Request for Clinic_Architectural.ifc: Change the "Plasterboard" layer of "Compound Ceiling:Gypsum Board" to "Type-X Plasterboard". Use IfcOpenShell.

First a look at what the model holds.

```python
import ifcopenshell
import ifcopenshell.util.element

model = ifcopenshell.open("Clinic_Architectural.ifc")
print(model.schema)
for layer_set in model.by_type("IfcMaterialLayerSet"):
    if layer_set.LayerSetName == "Compound Ceiling:Gypsum Board":
        for layer in layer_set.MaterialLayers:
            print(layer.id(), layer.Material and layer.Material.Name, layer.LayerThickness, sep=" | ")
        print(len(ifcopenshell.util.element.get_elements_by_material(model, layer_set)), "elements and types use it")
print(sorted(m.Name for m in model.by_type("IfcMaterial") if m.Name)[:60])
```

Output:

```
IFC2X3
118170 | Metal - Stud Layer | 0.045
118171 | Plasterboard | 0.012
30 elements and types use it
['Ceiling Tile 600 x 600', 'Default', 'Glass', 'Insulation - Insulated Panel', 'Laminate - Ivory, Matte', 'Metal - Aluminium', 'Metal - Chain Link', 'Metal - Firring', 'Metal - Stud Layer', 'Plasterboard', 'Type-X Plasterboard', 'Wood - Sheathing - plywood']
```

```python
import ifcopenshell
import ifcopenshell.api.material

model = ifcopenshell.open("Clinic_Architectural.ifc")

layer_set = next(s for s in model.by_type("IfcMaterialLayerSet") if s.LayerSetName == "Compound Ceiling:Gypsum Board")
layer = next(l for l in layer_set.MaterialLayers if l.Material and l.Material.Name == "Plasterboard")
material = next(m for m in model.by_type("IfcMaterial") if m.Name == "Type-X Plasterboard")

# Point this one layer at the other material; renaming the old one would change it everywhere.
ifcopenshell.api.material.edit_layer(model, layer=layer, attributes={}, material=material)

print([l.Material.Name if l.Material else None for l in layer_set.MaterialLayers])

model.write("Clinic_Architectural_v2.ifc")
```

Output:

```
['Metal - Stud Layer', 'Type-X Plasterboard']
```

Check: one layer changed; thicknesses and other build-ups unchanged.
